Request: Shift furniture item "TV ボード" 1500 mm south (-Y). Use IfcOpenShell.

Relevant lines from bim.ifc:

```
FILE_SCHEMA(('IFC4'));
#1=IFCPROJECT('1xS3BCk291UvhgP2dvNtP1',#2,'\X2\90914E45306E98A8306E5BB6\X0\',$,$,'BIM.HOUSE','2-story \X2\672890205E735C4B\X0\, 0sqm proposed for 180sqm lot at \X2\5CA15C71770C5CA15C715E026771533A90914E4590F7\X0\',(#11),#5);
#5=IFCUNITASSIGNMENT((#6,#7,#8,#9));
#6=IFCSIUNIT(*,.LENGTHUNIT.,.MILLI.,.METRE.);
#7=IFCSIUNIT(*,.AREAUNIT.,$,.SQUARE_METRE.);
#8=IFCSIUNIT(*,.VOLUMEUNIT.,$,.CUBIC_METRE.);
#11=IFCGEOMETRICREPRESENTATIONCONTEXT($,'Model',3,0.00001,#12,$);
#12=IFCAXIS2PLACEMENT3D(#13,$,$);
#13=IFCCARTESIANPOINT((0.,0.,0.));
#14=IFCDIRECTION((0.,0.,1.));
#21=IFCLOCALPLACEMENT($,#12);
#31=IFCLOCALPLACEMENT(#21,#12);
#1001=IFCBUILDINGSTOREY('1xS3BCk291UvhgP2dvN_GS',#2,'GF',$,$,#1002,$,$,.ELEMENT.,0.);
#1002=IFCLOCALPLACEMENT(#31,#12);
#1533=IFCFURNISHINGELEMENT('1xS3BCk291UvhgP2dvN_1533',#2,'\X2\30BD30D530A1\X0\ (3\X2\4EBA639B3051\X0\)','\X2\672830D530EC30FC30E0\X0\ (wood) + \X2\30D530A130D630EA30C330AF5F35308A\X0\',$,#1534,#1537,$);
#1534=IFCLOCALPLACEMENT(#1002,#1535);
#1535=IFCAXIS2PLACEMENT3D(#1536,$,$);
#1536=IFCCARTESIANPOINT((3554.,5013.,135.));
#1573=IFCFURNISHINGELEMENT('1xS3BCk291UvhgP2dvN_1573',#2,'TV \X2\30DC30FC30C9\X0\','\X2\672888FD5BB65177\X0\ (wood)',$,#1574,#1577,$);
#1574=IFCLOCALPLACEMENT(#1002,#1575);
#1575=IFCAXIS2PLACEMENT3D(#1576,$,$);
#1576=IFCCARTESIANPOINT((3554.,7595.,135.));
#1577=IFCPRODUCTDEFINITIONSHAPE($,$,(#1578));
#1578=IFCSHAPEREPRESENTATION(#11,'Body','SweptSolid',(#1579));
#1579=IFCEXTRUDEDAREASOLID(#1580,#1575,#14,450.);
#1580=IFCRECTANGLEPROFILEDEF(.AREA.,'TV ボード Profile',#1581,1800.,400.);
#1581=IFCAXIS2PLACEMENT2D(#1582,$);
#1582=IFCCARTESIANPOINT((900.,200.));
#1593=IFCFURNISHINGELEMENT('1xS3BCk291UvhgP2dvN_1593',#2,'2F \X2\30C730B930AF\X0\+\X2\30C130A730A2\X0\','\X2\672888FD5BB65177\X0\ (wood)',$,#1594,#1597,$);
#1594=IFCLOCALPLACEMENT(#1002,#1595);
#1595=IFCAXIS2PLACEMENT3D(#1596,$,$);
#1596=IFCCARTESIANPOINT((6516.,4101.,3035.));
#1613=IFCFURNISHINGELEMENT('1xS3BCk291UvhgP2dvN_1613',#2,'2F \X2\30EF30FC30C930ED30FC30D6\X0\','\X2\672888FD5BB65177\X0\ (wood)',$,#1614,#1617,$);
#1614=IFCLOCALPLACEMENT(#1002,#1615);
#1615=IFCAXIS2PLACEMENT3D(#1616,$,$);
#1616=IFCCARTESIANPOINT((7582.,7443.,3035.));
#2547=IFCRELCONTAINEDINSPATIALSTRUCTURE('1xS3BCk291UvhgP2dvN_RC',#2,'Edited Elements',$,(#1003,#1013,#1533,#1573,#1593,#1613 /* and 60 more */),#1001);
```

```python
import ifcopenshell
import ifcopenshell.api.geometry
import ifcopenshell.util.placement
import ifcopenshell.util.unit

model = ifcopenshell.open("bim.ifc")
unit_scale = ifcopenshell.util.unit.calculate_unit_scale(model)

item = model.by_guid("1xS3BCk291UvhgP2dvN_1573")
matrix = ifcopenshell.util.placement.get_local_placement(item.ObjectPlacement)
matrix[1, 3] -= 1.5 / unit_scale
ifcopenshell.api.geometry.edit_object_placement(model, product=item, matrix=matrix, is_si=False)

print(ifcopenshell.util.placement.get_local_placement(item.ObjectPlacement).round(3) + 0.0)

model.write("bim_v2.ifc")
```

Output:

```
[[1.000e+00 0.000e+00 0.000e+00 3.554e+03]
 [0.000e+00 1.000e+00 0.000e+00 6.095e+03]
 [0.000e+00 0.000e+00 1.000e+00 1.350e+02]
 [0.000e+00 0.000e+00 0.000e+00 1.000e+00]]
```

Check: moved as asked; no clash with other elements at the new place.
